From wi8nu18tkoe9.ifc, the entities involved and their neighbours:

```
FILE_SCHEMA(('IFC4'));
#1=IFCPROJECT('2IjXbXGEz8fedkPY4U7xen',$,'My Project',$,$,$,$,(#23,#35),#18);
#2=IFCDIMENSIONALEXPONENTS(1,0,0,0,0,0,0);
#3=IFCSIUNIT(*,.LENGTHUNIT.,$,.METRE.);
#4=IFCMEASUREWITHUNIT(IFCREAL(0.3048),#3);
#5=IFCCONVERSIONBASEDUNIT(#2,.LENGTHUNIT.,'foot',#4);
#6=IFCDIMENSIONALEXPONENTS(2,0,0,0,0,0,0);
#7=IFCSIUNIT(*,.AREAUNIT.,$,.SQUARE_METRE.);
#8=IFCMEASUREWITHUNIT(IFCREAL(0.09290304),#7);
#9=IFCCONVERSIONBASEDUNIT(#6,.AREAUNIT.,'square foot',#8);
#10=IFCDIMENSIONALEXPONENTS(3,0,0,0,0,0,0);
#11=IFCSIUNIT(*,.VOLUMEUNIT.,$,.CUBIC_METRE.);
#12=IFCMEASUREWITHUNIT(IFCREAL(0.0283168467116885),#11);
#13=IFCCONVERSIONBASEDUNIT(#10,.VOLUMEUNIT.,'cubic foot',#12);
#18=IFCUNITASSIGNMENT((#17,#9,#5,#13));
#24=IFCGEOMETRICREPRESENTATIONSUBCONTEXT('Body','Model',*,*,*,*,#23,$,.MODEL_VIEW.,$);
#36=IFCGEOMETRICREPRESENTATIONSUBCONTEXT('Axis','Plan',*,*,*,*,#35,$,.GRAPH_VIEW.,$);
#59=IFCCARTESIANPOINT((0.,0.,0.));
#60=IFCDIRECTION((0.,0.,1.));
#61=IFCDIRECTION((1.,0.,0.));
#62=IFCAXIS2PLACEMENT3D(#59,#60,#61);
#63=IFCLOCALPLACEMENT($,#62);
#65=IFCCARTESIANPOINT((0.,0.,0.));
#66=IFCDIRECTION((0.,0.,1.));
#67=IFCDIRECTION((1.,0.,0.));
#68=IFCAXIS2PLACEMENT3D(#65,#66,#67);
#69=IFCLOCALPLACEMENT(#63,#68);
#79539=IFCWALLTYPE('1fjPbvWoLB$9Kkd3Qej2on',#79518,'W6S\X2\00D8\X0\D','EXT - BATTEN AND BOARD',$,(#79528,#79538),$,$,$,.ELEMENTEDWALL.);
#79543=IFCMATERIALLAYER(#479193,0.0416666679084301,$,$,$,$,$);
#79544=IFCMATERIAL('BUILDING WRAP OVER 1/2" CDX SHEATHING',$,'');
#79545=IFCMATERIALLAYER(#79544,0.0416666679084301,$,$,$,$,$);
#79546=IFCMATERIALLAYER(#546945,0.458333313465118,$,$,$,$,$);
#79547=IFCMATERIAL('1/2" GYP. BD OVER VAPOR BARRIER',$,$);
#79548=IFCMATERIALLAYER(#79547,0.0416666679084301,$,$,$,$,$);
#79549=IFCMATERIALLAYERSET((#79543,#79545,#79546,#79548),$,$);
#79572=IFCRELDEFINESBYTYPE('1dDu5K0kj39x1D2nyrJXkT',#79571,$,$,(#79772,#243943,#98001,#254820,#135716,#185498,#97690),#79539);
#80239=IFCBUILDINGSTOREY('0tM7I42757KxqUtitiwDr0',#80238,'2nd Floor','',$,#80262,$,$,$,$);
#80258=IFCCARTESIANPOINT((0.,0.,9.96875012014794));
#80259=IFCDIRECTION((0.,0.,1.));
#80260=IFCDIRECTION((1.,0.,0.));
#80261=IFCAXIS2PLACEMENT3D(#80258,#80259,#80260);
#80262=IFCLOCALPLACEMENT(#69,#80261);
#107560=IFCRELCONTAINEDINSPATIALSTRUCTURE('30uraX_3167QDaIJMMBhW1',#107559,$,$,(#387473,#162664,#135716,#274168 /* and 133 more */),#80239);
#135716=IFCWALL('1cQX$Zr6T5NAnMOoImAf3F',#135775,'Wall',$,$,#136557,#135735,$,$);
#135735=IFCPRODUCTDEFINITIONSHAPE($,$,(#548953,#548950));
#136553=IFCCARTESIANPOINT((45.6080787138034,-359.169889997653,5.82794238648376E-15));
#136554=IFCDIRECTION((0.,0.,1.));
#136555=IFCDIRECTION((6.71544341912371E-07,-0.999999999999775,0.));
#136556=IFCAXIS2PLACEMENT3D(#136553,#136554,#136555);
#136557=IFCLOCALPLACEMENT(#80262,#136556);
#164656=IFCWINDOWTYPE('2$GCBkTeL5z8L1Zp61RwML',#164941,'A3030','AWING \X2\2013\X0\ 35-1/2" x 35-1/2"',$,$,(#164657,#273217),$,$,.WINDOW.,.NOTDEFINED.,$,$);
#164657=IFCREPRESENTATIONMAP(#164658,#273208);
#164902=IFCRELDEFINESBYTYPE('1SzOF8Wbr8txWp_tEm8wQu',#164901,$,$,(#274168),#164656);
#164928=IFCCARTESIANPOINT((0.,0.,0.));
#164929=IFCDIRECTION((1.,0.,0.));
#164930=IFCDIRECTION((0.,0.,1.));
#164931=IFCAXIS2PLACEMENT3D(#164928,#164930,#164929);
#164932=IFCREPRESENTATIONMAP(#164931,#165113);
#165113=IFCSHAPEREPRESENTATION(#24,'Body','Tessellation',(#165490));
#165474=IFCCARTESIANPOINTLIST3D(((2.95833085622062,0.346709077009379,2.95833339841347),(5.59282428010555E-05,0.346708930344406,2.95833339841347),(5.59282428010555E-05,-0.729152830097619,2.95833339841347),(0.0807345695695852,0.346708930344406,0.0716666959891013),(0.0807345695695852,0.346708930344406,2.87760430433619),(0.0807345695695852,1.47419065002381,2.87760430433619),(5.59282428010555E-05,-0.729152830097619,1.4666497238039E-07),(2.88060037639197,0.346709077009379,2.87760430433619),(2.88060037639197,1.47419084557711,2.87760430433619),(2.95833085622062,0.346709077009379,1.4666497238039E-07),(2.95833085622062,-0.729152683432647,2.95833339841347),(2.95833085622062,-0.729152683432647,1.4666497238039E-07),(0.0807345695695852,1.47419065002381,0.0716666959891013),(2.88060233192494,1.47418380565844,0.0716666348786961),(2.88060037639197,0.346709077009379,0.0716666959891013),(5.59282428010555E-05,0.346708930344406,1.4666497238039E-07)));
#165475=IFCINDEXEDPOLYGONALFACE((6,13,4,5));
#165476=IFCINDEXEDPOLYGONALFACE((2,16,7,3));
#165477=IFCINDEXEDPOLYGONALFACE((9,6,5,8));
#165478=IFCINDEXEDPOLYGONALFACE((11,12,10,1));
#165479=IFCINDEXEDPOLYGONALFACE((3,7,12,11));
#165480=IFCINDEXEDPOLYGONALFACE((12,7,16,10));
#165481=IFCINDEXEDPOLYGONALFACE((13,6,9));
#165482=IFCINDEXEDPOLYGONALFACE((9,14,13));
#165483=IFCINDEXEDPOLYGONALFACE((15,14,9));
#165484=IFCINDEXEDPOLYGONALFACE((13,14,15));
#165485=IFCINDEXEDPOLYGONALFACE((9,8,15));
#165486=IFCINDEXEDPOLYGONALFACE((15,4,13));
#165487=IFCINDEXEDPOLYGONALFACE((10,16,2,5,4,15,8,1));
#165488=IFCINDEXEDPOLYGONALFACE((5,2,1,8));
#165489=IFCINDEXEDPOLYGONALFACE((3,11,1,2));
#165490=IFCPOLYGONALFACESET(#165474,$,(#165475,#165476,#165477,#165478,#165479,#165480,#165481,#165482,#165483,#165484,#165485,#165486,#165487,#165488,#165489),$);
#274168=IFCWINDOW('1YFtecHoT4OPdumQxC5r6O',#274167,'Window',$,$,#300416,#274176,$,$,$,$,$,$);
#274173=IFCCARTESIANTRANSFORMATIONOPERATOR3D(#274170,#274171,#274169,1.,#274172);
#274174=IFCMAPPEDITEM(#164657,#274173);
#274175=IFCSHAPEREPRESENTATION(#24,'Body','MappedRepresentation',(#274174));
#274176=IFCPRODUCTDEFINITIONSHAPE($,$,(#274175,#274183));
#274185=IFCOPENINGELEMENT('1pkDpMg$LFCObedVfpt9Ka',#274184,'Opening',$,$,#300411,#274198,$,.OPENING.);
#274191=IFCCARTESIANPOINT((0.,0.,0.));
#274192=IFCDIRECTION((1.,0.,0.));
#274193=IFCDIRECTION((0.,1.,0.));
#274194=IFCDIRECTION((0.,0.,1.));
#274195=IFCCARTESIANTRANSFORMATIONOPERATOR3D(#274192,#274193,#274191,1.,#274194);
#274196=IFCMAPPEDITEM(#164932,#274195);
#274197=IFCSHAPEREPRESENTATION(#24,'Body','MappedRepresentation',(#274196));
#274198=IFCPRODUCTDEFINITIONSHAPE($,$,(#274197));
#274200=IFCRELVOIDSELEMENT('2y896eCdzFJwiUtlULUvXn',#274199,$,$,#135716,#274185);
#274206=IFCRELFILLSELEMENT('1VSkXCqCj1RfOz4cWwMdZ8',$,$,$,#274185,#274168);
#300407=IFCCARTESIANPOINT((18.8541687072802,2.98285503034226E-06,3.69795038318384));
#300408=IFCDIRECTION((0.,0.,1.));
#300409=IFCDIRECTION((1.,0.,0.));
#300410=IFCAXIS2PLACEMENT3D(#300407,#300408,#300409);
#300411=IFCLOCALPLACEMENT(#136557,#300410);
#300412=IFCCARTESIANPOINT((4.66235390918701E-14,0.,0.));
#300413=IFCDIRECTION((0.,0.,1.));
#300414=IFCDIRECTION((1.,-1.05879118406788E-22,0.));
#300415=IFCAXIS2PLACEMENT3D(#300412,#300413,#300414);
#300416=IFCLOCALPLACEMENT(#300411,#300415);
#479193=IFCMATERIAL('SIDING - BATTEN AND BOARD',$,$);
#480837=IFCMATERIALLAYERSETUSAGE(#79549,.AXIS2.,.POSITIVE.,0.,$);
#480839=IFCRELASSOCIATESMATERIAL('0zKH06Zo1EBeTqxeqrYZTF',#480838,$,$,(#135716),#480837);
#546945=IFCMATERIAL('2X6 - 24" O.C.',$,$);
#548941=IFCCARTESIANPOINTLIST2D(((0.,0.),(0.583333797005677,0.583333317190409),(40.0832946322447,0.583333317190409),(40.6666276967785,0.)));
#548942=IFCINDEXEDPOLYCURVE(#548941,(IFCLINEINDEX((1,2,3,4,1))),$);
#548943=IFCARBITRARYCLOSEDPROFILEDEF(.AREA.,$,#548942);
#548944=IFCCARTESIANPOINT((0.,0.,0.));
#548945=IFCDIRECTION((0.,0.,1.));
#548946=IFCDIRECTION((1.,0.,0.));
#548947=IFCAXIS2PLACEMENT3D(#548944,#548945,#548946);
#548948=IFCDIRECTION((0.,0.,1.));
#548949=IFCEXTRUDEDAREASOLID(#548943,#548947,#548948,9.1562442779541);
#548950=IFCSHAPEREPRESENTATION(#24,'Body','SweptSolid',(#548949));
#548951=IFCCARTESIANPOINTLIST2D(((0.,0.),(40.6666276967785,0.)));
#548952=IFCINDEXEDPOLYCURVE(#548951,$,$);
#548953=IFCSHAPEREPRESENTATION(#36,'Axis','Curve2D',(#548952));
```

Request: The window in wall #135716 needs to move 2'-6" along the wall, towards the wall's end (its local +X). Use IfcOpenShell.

```python
import ifcopenshell
import ifcopenshell.api.geometry
import ifcopenshell.util.placement
import ifcopenshell.util.unit

model = ifcopenshell.open("wi8nu18tkoe9.ifc")
unit_scale = ifcopenshell.util.unit.calculate_unit_scale(model)

window = model.by_guid("1YFtecHoT4OPdumQxC5r6O")
opening = window.FillsVoids[0].RelatingOpeningElement
wall = opening.VoidsElements[0].RelatingBuildingElement

wall_matrix = ifcopenshell.util.placement.get_local_placement(wall.ObjectPlacement)
shift = wall_matrix[:3, 0] * 30 * 0.0254 / unit_scale
before = ifcopenshell.util.placement.get_local_placement(window.ObjectPlacement)[:3, 3].copy()

# The window is placed relative to its opening, so it follows when the opening moves.
matrix = ifcopenshell.util.placement.get_local_placement(opening.ObjectPlacement)
matrix[:3, 3] += shift
ifcopenshell.api.geometry.edit_object_placement(
    model, product=opening, matrix=matrix, is_si=False, should_transform_children=True
)

after = ifcopenshell.util.placement.get_local_placement(window.ObjectPlacement)[:3, 3]
print("window moved by", (after - before).round(3) + 0.0)

model.write("wi8nu18tkoe9_v2.ifc")
```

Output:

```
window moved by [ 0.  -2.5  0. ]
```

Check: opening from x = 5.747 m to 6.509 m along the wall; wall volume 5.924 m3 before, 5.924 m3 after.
